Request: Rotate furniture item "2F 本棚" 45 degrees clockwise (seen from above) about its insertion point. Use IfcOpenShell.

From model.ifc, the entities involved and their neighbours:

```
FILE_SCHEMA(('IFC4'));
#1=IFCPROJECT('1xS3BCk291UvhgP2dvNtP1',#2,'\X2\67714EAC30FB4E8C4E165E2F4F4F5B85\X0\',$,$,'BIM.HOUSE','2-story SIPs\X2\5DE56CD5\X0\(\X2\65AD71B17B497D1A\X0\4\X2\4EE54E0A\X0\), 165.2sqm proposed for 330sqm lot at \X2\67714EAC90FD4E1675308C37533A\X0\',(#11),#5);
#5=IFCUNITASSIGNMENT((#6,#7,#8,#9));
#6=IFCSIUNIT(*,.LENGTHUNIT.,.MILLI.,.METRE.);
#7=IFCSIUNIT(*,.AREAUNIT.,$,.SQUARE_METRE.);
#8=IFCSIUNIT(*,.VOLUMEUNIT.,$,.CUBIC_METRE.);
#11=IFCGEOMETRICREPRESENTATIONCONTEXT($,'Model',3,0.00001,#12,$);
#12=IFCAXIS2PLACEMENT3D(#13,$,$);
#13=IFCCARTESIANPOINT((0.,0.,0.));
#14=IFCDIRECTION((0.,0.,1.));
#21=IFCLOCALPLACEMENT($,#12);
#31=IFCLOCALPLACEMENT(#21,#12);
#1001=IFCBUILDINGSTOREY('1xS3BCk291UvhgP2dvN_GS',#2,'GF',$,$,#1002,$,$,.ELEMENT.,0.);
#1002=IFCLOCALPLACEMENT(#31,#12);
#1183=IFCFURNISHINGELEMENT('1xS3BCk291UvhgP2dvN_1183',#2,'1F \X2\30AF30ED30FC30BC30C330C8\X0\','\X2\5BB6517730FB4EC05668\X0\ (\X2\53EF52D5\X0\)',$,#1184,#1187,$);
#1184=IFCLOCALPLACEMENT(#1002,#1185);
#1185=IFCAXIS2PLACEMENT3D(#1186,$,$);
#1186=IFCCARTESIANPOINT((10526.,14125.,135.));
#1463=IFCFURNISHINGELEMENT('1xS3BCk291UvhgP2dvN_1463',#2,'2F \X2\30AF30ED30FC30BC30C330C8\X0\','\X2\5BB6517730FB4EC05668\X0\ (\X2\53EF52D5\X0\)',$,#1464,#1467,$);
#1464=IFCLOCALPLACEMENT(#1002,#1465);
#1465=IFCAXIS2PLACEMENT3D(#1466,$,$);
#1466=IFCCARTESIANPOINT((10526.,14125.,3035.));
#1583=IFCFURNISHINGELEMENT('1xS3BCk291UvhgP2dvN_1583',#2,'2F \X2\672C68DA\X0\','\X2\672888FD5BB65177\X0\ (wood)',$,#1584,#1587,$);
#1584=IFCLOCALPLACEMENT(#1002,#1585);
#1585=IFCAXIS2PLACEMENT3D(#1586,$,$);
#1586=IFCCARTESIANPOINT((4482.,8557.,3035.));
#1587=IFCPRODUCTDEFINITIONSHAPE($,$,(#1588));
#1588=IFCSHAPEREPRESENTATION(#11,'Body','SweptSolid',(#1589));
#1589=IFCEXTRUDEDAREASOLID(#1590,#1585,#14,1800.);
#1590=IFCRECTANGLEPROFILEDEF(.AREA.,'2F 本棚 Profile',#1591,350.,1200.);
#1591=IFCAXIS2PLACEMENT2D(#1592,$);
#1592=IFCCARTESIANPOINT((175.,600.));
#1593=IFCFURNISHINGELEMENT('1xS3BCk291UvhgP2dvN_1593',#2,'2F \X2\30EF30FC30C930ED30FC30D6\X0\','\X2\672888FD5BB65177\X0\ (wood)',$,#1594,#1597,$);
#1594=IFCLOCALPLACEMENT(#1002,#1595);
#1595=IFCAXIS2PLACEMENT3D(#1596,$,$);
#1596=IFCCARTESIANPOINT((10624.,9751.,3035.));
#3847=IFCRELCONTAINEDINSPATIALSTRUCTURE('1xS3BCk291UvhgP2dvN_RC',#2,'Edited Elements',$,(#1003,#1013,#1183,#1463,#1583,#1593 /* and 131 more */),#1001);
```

```python
import ifcopenshell
import ifcopenshell.api.geometry
import ifcopenshell.util.placement

model = ifcopenshell.open("model.ifc")

item = model.by_guid("1xS3BCk291UvhgP2dvN_1583")
matrix = ifcopenshell.util.placement.get_local_placement(item.ObjectPlacement)
matrix = matrix @ ifcopenshell.util.placement.rotation(-45, "Z")
ifcopenshell.api.geometry.edit_object_placement(model, product=item, matrix=matrix, is_si=False)

print(ifcopenshell.util.placement.get_local_placement(item.ObjectPlacement).round(3) + 0.0)

model.write("model-out.ifc")
```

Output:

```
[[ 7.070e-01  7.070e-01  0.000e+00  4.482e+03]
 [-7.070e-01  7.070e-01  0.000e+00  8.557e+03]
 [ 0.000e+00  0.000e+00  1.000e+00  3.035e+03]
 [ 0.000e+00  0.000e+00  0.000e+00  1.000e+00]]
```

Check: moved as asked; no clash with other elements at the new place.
